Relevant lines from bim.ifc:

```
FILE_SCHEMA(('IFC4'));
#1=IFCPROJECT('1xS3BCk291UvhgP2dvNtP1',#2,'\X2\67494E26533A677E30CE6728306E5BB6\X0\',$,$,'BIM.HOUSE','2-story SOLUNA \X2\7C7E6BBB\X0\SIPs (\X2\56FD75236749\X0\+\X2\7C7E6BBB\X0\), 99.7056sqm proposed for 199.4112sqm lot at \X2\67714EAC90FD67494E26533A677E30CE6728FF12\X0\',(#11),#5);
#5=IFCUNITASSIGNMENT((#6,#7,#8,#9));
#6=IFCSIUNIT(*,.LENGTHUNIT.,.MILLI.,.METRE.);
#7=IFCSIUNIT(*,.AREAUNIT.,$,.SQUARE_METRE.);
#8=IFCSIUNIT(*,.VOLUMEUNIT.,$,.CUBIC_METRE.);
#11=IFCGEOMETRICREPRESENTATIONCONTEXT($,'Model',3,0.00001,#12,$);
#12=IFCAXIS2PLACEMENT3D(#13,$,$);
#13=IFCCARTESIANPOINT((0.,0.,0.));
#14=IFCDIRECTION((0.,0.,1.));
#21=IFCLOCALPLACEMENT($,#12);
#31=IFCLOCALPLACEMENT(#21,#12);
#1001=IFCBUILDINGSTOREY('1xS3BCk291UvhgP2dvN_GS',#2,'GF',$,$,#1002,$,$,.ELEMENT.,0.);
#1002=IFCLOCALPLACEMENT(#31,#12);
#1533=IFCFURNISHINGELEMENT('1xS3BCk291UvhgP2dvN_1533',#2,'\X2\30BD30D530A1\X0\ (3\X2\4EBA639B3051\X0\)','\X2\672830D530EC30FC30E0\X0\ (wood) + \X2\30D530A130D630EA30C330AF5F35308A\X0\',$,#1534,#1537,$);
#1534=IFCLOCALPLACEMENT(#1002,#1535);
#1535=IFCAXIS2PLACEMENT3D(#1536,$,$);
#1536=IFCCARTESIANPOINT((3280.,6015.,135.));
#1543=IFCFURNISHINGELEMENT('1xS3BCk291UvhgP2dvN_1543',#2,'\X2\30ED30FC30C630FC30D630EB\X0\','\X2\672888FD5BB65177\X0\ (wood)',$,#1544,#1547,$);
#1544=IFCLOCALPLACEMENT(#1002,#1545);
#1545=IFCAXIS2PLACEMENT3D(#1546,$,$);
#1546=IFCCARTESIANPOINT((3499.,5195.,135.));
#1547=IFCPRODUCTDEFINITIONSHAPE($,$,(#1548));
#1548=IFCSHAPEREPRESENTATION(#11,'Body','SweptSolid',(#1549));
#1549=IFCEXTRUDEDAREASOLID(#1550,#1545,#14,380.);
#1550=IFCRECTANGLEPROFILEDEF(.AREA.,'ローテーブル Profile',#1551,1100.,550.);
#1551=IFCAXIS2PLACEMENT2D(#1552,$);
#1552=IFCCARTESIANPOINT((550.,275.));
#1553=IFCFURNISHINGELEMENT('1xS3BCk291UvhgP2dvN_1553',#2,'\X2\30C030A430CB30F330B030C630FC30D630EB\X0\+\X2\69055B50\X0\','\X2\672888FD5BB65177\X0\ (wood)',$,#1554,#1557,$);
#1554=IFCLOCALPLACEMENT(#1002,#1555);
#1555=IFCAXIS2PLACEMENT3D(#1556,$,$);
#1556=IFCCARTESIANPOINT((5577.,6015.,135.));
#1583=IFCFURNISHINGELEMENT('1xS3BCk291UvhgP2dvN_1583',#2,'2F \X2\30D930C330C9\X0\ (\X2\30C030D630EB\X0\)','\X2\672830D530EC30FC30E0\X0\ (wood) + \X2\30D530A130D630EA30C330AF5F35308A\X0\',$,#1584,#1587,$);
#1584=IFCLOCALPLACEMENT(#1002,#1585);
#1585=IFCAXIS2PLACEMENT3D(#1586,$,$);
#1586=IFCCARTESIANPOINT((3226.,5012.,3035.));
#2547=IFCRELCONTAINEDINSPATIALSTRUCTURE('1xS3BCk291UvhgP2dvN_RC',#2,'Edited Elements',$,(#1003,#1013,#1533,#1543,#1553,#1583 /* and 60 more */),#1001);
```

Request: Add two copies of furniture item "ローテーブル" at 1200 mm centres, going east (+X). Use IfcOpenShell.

```python
import numpy as np
import ifcopenshell
import ifcopenshell.api.geometry
import ifcopenshell.api.root
import ifcopenshell.util.element
import ifcopenshell.util.placement
import ifcopenshell.util.unit

model = ifcopenshell.open("bim.ifc")
unit_scale = ifcopenshell.util.unit.calculate_unit_scale(model)


def reuse_history(source, copy):
    """copy_class also copies each property set's owner history, people and application; keep the originals."""
    for rel in copy.IsDefinedBy:
        if rel.is_a("IfcRelDefinesByProperties") and (history := rel.RelatingPropertyDefinition.OwnerHistory):
            rel.RelatingPropertyDefinition.OwnerHistory = source.OwnerHistory
            ifcopenshell.util.element.remove_deep2(model, history)


source = model.by_guid("1xS3BCk291UvhgP2dvN_1543")
base = ifcopenshell.util.placement.get_local_placement(source.ObjectPlacement)
step = np.array([1.0, 0.0, 0.0]) * 1.2 / unit_scale

for i in range(1, 3):
    copy = ifcopenshell.api.root.copy_class(model, product=source)
    copy.Representation = ifcopenshell.util.element.copy_deep(
        model, source.Representation, exclude=["IfcGeometricRepresentationContext", "IfcRepresentationMap"]
    )
    reuse_history(source, copy)
    matrix = base.copy()
    matrix[:3, 3] += i * step
    print("added at", matrix[:3, 3].round(3) + 0.0)
    ifcopenshell.api.geometry.edit_object_placement(model, product=copy, matrix=matrix, is_si=False)

model.write("bim_rev.ifc")
```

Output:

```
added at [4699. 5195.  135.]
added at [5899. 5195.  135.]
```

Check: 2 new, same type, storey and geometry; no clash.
